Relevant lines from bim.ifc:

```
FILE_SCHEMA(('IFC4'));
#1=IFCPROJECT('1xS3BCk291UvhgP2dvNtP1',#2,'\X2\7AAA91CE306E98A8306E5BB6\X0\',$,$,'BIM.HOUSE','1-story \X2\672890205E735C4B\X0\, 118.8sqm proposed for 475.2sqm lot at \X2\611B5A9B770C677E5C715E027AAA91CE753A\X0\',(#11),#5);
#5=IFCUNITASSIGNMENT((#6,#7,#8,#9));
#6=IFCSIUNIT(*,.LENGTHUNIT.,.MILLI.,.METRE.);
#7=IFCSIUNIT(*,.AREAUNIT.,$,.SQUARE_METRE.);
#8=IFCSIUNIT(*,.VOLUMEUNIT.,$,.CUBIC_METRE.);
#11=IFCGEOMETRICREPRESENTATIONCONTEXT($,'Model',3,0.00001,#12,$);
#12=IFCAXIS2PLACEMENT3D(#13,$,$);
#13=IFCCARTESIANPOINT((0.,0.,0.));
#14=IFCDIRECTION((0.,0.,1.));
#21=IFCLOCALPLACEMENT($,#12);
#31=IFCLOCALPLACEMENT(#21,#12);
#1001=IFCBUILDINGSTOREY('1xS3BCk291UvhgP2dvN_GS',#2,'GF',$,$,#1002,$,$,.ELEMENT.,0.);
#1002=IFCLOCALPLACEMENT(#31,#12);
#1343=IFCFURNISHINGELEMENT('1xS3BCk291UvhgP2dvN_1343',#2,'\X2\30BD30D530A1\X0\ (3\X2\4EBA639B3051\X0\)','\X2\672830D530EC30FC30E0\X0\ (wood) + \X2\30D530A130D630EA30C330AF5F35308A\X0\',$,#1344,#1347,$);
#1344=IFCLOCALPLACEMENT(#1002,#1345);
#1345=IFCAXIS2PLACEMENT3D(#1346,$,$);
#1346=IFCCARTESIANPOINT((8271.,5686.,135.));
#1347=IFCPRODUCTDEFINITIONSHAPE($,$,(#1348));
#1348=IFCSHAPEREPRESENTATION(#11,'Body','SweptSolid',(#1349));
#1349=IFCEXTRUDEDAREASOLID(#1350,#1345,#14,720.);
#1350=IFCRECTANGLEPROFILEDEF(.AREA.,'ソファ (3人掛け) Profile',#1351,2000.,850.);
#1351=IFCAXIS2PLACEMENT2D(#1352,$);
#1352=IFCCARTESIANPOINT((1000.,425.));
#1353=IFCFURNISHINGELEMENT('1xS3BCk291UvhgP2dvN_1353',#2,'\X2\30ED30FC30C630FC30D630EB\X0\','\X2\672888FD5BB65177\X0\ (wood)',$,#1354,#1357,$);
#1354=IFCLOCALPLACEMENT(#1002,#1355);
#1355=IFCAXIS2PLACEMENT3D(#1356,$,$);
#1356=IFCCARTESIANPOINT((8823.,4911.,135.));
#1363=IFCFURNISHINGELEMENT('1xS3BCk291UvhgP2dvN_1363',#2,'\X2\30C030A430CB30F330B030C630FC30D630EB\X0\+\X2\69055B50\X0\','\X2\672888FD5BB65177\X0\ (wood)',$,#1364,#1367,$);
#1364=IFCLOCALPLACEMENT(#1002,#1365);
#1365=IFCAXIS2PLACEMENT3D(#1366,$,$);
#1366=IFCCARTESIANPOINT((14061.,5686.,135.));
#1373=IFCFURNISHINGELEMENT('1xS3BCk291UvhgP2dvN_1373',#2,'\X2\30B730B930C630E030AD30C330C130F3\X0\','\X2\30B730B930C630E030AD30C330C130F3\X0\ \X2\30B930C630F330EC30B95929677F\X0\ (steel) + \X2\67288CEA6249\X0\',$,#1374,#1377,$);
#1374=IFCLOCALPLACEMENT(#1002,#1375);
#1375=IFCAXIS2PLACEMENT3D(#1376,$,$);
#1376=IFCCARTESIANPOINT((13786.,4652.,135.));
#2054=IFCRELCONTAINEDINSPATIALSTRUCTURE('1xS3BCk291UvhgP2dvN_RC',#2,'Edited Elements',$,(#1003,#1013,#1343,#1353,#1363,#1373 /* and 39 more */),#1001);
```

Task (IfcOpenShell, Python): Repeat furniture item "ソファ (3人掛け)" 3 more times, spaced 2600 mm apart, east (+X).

```python
import numpy as np
import ifcopenshell
import ifcopenshell.api.geometry
import ifcopenshell.api.root
import ifcopenshell.util.element
import ifcopenshell.util.placement
import ifcopenshell.util.unit

model = ifcopenshell.open("bim.ifc")
unit_scale = ifcopenshell.util.unit.calculate_unit_scale(model)


def reuse_history(source, copy):
    """copy_class also copies each property set's owner history, people and application; keep the originals."""
    for rel in copy.IsDefinedBy:
        if rel.is_a("IfcRelDefinesByProperties") and (history := rel.RelatingPropertyDefinition.OwnerHistory):
            rel.RelatingPropertyDefinition.OwnerHistory = source.OwnerHistory
            ifcopenshell.util.element.remove_deep2(model, history)


source = model.by_guid("1xS3BCk291UvhgP2dvN_1343")
base = ifcopenshell.util.placement.get_local_placement(source.ObjectPlacement)
step = np.array([1.0, 0.0, 0.0]) * 2.6 / unit_scale

for i in range(1, 4):
    copy = ifcopenshell.api.root.copy_class(model, product=source)
    copy.Representation = ifcopenshell.util.element.copy_deep(
        model, source.Representation, exclude=["IfcGeometricRepresentationContext", "IfcRepresentationMap"]
    )
    reuse_history(source, copy)
    matrix = base.copy()
    matrix[:3, 3] += i * step
    print("added at", matrix[:3, 3].round(3) + 0.0)
    ifcopenshell.api.geometry.edit_object_placement(model, product=copy, matrix=matrix, is_si=False)

model.write("bim_edited.ifc")
```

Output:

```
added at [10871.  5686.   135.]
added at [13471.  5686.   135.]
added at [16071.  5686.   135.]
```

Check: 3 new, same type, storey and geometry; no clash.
